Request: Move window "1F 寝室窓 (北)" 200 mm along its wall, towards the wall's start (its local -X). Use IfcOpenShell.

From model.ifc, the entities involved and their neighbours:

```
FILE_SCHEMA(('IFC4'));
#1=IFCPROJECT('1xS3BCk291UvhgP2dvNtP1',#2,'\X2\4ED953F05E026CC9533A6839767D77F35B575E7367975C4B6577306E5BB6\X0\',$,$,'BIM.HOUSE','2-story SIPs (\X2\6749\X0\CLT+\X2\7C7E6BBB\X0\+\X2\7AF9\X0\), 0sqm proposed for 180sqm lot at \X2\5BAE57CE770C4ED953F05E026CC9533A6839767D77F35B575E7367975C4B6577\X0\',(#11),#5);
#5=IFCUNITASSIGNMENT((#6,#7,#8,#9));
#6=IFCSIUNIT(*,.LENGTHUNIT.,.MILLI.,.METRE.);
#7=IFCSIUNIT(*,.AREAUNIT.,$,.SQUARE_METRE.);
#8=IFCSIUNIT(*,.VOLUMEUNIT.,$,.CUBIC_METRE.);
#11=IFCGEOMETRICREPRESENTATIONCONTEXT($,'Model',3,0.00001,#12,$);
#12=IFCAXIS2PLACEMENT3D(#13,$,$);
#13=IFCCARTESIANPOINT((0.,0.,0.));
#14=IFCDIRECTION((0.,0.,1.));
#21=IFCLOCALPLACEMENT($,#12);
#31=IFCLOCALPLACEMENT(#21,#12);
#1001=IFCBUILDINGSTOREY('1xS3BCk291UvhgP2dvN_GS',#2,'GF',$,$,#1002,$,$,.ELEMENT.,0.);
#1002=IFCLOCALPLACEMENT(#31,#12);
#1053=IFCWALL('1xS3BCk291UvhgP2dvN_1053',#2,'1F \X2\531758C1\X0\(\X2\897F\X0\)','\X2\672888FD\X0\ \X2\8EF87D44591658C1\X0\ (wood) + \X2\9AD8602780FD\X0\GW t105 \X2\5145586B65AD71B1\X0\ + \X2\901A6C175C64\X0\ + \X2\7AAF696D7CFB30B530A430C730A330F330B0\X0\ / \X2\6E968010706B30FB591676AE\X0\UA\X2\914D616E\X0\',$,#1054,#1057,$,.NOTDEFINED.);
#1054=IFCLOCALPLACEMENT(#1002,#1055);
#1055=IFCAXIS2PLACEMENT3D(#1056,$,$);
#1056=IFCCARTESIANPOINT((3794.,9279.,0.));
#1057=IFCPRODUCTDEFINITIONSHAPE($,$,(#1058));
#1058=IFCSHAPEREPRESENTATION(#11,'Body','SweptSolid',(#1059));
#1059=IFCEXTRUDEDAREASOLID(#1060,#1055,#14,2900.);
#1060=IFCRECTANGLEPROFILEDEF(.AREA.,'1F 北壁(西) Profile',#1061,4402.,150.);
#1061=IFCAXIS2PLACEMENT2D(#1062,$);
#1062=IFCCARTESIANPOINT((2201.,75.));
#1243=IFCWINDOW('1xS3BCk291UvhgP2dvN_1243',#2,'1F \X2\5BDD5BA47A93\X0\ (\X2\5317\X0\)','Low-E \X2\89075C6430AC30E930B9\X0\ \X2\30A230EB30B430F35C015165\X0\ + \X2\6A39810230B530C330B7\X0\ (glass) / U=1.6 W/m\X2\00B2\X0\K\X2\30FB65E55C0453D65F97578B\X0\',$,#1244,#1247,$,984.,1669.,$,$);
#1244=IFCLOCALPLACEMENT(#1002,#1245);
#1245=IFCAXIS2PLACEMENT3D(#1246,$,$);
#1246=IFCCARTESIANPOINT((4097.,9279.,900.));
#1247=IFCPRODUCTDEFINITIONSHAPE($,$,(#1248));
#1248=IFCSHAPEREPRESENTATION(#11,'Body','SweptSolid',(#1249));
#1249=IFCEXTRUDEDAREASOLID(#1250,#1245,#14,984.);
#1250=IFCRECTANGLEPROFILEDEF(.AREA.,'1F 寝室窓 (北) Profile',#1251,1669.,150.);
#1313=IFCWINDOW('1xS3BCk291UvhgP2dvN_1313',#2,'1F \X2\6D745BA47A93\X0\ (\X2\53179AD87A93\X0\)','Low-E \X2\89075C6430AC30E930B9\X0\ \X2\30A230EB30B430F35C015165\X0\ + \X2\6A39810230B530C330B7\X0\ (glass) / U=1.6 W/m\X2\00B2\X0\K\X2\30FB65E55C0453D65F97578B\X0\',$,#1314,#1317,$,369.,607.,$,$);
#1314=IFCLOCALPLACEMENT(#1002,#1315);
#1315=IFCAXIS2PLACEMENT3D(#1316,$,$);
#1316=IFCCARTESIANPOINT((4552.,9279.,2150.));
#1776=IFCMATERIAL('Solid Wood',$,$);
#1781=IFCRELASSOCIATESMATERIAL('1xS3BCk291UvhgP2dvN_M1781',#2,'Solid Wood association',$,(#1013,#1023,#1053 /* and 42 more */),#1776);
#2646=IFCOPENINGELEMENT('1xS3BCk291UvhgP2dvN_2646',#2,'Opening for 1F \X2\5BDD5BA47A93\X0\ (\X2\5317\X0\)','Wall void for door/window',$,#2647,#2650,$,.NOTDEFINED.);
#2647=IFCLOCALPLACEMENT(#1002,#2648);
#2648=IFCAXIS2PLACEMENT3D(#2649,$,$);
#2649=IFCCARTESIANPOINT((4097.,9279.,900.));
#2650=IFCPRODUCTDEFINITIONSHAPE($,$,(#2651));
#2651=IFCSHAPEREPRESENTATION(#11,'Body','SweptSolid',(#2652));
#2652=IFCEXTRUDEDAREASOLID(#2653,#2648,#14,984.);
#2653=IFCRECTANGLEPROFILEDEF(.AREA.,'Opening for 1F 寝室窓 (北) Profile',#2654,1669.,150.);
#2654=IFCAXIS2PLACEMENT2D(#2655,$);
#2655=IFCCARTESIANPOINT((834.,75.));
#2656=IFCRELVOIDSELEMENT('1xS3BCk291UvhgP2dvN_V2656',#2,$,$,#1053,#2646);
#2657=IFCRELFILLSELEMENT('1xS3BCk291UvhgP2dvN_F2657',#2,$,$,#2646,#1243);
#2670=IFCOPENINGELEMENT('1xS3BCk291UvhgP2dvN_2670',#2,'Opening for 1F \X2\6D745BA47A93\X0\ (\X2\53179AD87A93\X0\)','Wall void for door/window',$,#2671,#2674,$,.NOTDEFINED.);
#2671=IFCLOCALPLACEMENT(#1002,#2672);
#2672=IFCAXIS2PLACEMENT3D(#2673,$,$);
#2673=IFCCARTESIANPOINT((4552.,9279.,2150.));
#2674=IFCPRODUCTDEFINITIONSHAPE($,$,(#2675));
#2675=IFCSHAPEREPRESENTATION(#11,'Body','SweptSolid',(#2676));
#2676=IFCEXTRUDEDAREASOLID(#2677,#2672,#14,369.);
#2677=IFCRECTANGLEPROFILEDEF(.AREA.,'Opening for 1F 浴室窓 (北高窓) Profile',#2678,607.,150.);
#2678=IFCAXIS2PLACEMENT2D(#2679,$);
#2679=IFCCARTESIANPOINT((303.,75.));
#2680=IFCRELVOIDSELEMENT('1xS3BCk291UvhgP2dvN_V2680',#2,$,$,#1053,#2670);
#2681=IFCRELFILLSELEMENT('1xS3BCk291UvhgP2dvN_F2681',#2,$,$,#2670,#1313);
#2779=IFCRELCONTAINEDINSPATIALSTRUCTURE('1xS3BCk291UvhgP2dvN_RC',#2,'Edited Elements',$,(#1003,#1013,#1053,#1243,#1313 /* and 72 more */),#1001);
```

```python
import ifcopenshell
import ifcopenshell.api.geometry
import ifcopenshell.util.placement
import ifcopenshell.util.unit

model = ifcopenshell.open("model.ifc")
unit_scale = ifcopenshell.util.unit.calculate_unit_scale(model)

window = model.by_guid("1xS3BCk291UvhgP2dvN_1243")
opening = window.FillsVoids[0].RelatingOpeningElement
wall = opening.VoidsElements[0].RelatingBuildingElement

wall_matrix = ifcopenshell.util.placement.get_local_placement(wall.ObjectPlacement)
shift = wall_matrix[:3, 0] * -0.2 / unit_scale
before = ifcopenshell.util.placement.get_local_placement(window.ObjectPlacement)[:3, 3].copy()

# The window is not placed relative to its opening, so move both.
for product in (opening, window):
    matrix = ifcopenshell.util.placement.get_local_placement(product.ObjectPlacement)
    matrix[:3, 3] += shift
    ifcopenshell.api.geometry.edit_object_placement(model, product=product, matrix=matrix, is_si=False)

after = ifcopenshell.util.placement.get_local_placement(window.ObjectPlacement)[:3, 3]
print("window moved by", (after - before).round(3) + 0.0)

model.write("model_edited.ifc")
```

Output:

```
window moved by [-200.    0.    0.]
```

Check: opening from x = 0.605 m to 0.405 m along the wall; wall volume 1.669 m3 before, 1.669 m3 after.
